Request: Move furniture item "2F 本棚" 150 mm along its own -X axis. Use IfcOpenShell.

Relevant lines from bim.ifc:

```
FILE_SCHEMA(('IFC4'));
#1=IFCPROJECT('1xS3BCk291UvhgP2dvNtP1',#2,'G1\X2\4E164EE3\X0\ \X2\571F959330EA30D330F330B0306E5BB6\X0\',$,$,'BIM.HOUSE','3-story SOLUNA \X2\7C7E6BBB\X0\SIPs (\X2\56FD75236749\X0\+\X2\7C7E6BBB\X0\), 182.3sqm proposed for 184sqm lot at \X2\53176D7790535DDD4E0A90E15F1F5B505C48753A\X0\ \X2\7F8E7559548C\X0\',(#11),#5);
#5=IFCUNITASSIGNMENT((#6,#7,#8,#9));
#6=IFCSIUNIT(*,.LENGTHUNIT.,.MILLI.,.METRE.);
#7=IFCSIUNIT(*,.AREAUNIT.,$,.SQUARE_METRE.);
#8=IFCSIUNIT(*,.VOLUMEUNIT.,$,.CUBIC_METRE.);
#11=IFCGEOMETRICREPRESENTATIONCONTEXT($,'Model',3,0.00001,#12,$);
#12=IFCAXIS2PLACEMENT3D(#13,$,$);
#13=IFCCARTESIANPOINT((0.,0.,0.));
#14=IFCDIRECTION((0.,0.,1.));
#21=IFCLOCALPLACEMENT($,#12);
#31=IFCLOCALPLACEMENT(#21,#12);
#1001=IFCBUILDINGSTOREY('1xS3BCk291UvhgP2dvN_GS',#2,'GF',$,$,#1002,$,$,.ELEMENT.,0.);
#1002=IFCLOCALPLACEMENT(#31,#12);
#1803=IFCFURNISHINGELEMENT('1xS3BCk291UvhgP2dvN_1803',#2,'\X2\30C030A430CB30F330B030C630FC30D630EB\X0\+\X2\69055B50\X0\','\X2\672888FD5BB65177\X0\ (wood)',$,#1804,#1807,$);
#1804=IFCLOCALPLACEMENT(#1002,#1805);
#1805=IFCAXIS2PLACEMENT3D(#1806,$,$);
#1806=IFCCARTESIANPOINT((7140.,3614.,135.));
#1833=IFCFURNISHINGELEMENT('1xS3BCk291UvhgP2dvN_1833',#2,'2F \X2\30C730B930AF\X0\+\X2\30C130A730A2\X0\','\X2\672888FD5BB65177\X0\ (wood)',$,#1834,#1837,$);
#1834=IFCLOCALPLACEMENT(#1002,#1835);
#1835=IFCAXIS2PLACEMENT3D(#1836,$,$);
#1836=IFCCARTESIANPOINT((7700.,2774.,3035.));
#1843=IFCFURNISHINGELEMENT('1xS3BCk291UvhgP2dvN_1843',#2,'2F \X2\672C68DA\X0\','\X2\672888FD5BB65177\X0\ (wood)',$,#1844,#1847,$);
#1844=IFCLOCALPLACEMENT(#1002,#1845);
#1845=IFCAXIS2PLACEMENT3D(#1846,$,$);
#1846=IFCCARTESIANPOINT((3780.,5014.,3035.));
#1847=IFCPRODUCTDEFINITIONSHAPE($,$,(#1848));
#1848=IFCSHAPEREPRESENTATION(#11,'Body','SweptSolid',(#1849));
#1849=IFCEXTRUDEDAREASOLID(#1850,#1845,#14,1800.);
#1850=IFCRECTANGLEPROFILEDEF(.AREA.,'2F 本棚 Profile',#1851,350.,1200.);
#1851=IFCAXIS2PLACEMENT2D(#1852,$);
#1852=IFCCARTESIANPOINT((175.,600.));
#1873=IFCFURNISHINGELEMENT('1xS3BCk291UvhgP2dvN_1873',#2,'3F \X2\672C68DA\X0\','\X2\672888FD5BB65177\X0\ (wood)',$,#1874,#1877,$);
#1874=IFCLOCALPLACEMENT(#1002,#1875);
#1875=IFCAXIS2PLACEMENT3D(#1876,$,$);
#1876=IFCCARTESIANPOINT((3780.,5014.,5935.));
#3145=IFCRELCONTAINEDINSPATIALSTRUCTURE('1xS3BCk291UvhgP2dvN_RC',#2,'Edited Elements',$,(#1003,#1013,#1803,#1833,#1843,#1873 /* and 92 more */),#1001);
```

```python
import ifcopenshell
import ifcopenshell.api.geometry
import ifcopenshell.util.placement

model = ifcopenshell.open("bim.ifc")

item = model.by_guid("1xS3BCk291UvhgP2dvN_1843")
matrix = ifcopenshell.util.placement.get_local_placement(item.ObjectPlacement)
matrix[:3, 3] -= matrix[:3, 0] * 150.0
ifcopenshell.api.geometry.edit_object_placement(model, product=item, matrix=matrix, is_si=False)

print(ifcopenshell.util.placement.get_local_placement(item.ObjectPlacement).round(3) + 0.0)

model.write("bim-out.ifc")
```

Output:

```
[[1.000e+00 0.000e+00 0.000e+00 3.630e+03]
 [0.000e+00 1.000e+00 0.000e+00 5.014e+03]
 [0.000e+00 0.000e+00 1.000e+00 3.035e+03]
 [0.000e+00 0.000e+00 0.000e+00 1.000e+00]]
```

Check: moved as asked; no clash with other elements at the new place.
